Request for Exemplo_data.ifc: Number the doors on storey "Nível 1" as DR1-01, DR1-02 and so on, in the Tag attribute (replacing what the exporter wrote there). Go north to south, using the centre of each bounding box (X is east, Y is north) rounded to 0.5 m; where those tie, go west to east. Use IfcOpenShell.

First a look at what the model holds.

```python
import ifcopenshell
import ifcopenshell.util.element
import ifcopenshell.util.placement

model = ifcopenshell.open("Exemplo_data.ifc")
print(model.schema)
storey = next(s for s in model.by_type("IfcBuildingStorey") if s.Name == "Nível 1")
doors = [e for e in ifcopenshell.util.element.get_decomposition(storey) if e.is_a("IfcDoor")]
for e in sorted(doors, key=lambda e: e.id()):
    origin = ifcopenshell.util.placement.get_local_placement(e.ObjectPlacement)[:3, 3]
    print(e.id(), e.Tag, e.Name, origin.round(2) + 0.0, sep=" | ")
```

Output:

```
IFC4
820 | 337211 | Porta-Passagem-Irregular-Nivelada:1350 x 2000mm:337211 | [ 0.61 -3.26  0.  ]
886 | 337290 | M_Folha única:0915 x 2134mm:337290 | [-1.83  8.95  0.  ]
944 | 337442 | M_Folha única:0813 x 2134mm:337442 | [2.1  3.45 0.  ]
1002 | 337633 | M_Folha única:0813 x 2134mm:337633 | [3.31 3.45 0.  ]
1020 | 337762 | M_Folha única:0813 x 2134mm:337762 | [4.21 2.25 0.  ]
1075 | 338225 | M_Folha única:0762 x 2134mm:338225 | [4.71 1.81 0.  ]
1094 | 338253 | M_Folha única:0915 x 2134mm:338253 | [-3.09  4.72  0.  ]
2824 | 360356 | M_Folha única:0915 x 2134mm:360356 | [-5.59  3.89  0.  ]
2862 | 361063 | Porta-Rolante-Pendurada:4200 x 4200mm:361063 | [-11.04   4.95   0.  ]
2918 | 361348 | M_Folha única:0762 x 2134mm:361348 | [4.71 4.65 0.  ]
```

```python
import ifcopenshell
import ifcopenshell.geom
import ifcopenshell.util.element
import ifcopenshell.util.shape

model = ifcopenshell.open("Exemplo_data.ifc")
settings = ifcopenshell.geom.settings()
settings.set("use-world-coords", True)


def centre(element):
    shape = ifcopenshell.geom.create_shape(settings, element)
    return ifcopenshell.util.shape.get_bbox_centroid(shape.geometry)


storey = next(s for s in model.by_type("IfcBuildingStorey") if s.Name == "Nível 1")
doors = [e for e in ifcopenshell.util.element.get_decomposition(storey) if e.is_a("IfcDoor")]

# Insertion points can sit at a corner or the storey origin, so sort by the geometry (in metres).
centres = {e: centre(e) for e in doors}
doors.sort(key=lambda e: (-round(centres[e][1] / 0.5), centres[e][0]))

for i, e in enumerate(doors, start=1):
    number = f"DR1-{i:02d}"
    e.Tag = number
    print(e.id(), number)

model.write("Exemplo_data_rev.ifc")
```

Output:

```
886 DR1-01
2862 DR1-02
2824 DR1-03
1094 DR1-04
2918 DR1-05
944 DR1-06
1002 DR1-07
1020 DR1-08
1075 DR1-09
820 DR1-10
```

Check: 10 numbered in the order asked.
